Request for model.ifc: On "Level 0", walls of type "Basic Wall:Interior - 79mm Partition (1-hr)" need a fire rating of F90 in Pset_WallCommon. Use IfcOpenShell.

First a look at what the model holds.

```python
import ifcopenshell
import ifcopenshell.util.element

model = ifcopenshell.open("model.ifc")
print(model.schema)
storey = next(s for s in model.by_type("IfcBuildingStorey") if s.Name == "Level 0")
walls = [e for e in ifcopenshell.util.element.get_decomposition(storey) if e.is_a("IfcWall")]
seen = {}
for e in walls:
    element_type = ifcopenshell.util.element.get_type(e)
    key = (element_type.Name if element_type != e and element_type else None, ifcopenshell.util.element.get_pset(e, "Pset_WallCommon", "FireRating"))
    seen[key] = seen.get(key, 0) + 1
for (name, value), count in sorted(seen.items(), key=str):
    print(count, "x", name, "|", value)
```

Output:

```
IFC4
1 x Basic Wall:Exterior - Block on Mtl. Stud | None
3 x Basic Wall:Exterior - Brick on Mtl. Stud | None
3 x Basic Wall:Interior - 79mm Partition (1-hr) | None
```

```python
import ifcopenshell
import ifcopenshell.api.pset
import ifcopenshell.util.element

model = ifcopenshell.open("model.ifc")

storey = next(s for s in model.by_type("IfcBuildingStorey") if s.Name == "Level 0")
walls = [e for e in ifcopenshell.util.element.get_decomposition(storey) if e.is_a("IfcWall")]

count = 0
for e in walls:
    element_type = ifcopenshell.util.element.get_type(e)
    if element_type in (None, e) or element_type.Name != "Basic Wall:Interior - 79mm Partition (1-hr)":
        continue
    # add_pset returns the element's existing set when there is one.
    pset = ifcopenshell.api.pset.add_pset(model, product=e, name="Pset_WallCommon")
    ifcopenshell.api.pset.edit_pset(model, pset=pset, properties={"FireRating": "F90"})
    count += 1

print(count, "walls updated")

model.write("model_v2.ifc")
```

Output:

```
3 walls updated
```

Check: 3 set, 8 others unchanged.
